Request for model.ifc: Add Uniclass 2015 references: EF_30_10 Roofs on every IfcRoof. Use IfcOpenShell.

First a look at what the model holds.

```python
import ifcopenshell

model = ifcopenshell.open("model.ifc")
print(model.schema)
print("classifications:", [c.Name for c in model.by_type("IfcClassification")])
for ifc_class in ("IfcDoor", "IfcRoof", "IfcStair", "IfcWall", "IfcWindow"):
    print(ifc_class, len(model.by_type(ifc_class)))
```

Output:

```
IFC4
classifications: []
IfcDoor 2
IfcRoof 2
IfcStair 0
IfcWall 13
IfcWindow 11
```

```python
import ifcopenshell
import ifcopenshell.api.classification

model = ifcopenshell.open("model.ifc")

system = ifcopenshell.api.classification.add_classification(model, classification="Uniclass 2015")

codes = {
    "IfcRoof": ("EF_30_10", "Roofs"),
}
for ifc_class, (code, name) in codes.items():
    products = model.by_type(ifc_class)
    ifcopenshell.api.classification.add_reference(
        model, products=products, classification=system, identification=code, name=name
    )
    print(code, len(products))

model.write("model_v2.ifc")
```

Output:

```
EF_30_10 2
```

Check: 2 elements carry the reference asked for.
